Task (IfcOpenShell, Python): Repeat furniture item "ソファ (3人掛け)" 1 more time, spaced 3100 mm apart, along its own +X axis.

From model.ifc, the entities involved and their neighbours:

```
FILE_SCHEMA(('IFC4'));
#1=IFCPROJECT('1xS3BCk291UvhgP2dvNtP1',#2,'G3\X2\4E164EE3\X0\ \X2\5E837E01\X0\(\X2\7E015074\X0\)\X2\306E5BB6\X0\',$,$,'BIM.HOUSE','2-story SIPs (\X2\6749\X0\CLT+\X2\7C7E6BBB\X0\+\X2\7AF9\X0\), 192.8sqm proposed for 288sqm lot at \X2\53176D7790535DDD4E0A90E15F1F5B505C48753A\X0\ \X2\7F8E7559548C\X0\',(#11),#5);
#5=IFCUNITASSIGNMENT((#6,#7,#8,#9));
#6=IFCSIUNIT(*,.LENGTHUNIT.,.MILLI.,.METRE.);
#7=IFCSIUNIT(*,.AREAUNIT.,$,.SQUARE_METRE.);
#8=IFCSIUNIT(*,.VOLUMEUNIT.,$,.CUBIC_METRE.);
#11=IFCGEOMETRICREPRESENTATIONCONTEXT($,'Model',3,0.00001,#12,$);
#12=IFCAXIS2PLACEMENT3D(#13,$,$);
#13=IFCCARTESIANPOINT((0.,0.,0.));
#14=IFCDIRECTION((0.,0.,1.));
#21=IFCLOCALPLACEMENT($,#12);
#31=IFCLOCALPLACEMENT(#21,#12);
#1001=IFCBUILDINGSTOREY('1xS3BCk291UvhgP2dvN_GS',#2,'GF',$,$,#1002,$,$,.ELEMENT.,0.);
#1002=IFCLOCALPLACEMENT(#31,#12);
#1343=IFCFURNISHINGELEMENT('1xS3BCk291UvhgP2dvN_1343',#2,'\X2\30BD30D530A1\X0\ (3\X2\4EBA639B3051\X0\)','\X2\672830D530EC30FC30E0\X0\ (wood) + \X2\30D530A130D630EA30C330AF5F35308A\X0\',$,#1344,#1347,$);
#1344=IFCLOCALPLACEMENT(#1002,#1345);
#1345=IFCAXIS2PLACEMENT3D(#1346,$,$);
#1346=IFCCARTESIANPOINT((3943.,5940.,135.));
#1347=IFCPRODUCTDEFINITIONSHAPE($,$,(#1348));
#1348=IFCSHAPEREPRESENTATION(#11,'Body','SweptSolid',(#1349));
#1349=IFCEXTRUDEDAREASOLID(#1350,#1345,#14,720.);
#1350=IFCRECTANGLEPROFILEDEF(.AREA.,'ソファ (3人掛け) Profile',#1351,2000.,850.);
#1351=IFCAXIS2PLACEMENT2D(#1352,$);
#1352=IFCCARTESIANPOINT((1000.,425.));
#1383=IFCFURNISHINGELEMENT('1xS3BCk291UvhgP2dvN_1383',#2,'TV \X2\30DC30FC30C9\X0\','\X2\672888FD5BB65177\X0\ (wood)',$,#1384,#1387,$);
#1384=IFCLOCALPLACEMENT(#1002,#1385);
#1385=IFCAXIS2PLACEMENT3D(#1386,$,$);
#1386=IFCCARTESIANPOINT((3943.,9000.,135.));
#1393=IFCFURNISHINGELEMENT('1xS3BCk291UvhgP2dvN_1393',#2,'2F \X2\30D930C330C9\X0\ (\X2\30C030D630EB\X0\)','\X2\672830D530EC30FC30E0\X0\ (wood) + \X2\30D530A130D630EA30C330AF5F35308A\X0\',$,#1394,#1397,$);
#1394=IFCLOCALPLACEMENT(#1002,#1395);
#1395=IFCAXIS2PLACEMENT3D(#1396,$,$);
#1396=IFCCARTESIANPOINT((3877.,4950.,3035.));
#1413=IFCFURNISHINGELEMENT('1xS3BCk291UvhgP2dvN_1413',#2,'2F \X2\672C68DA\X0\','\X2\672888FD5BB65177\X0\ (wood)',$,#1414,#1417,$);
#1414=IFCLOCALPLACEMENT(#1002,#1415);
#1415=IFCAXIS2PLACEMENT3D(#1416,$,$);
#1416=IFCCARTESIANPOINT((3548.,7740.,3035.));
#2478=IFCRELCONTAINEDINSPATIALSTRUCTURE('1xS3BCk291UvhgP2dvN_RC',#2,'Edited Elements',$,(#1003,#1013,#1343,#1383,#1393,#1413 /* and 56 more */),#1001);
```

```python
import ifcopenshell
import ifcopenshell.api.geometry
import ifcopenshell.api.root
import ifcopenshell.util.element
import ifcopenshell.util.placement
import ifcopenshell.util.unit

model = ifcopenshell.open("model.ifc")
unit_scale = ifcopenshell.util.unit.calculate_unit_scale(model)


def reuse_history(source, copy):
    """copy_class also copies each property set's owner history, people and application; keep the originals."""
    for rel in copy.IsDefinedBy:
        if rel.is_a("IfcRelDefinesByProperties") and (history := rel.RelatingPropertyDefinition.OwnerHistory):
            rel.RelatingPropertyDefinition.OwnerHistory = source.OwnerHistory
            ifcopenshell.util.element.remove_deep2(model, history)


source = model.by_guid("1xS3BCk291UvhgP2dvN_1343")
base = ifcopenshell.util.placement.get_local_placement(source.ObjectPlacement)
step = base[:3, 0] * 3.1 / unit_scale

for i in range(1, 2):
    copy = ifcopenshell.api.root.copy_class(model, product=source)
    copy.Representation = ifcopenshell.util.element.copy_deep(
        model, source.Representation, exclude=["IfcGeometricRepresentationContext", "IfcRepresentationMap"]
    )
    reuse_history(source, copy)
    matrix = base.copy()
    matrix[:3, 3] += i * step
    print("added at", matrix[:3, 3].round(3) + 0.0)
    ifcopenshell.api.geometry.edit_object_placement(model, product=copy, matrix=matrix, is_si=False)

model.write("model_rev.ifc")
```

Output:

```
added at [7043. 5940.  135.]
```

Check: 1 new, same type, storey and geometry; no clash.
